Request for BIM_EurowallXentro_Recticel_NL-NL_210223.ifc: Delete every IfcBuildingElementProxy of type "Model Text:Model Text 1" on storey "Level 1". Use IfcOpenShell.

First a look at what the model holds.

```python
import ifcopenshell
import ifcopenshell.util.element

model = ifcopenshell.open("BIM_EurowallXentro_Recticel_NL-NL_210223.ifc")
print(model.schema)
storey = next(s for s in model.by_type("IfcBuildingStorey") if s.Name == "Level 1")
proxies = [e for e in ifcopenshell.util.element.get_decomposition(storey) if e.is_a("IfcBuildingElementProxy")]
seen = {}
for e in proxies:
    element_type = ifcopenshell.util.element.get_type(e)
    name = element_type.Name if element_type not in (None, e) else None
    seen[name] = seen.get(name, 0) + 1
for name, count in sorted(seen.items(), key=str):
    print(count, "x", name)
```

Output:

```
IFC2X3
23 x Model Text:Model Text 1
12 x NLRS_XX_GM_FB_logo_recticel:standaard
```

```python
import ifcopenshell
import ifcopenshell.api.root
import ifcopenshell.util.element

model = ifcopenshell.open("BIM_EurowallXentro_Recticel_NL-NL_210223.ifc")

storey = next(s for s in model.by_type("IfcBuildingStorey") if s.Name == "Level 1")
proxies = [e for e in ifcopenshell.util.element.get_decomposition(storey) if e.is_a("IfcBuildingElementProxy")]
targets = [e for e in proxies if (t := ifcopenshell.util.element.get_type(e)) not in (None, e) and t.Name == "Model Text:Model Text 1"]

for e in targets:
    ifcopenshell.api.root.remove_product(model, product=e)
print(len(targets), "removed")

model.write("BIM_EurowallXentro_Recticel_NL-NL_210223-out.ifc")
```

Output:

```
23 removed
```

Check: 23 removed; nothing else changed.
